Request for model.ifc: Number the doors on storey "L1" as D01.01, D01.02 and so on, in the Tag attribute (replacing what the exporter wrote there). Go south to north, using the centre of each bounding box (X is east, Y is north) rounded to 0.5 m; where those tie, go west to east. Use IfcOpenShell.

First a look at what the model holds.

```python
import ifcopenshell
import ifcopenshell.util.element
import ifcopenshell.util.placement

model = ifcopenshell.open("model.ifc")
print(model.schema)
storey = next(s for s in model.by_type("IfcBuildingStorey") if s.Name == "L1")
doors = [e for e in ifcopenshell.util.element.get_decomposition(storey) if e.is_a("IfcDoor")]
for e in sorted(doors, key=lambda e: e.id()):
    origin = ifcopenshell.util.placement.get_local_placement(e.ObjectPlacement)[:3, 3]
    print(e.id(), e.Tag, e.Name, origin.round(2) + 0.0, sep=" | ")
```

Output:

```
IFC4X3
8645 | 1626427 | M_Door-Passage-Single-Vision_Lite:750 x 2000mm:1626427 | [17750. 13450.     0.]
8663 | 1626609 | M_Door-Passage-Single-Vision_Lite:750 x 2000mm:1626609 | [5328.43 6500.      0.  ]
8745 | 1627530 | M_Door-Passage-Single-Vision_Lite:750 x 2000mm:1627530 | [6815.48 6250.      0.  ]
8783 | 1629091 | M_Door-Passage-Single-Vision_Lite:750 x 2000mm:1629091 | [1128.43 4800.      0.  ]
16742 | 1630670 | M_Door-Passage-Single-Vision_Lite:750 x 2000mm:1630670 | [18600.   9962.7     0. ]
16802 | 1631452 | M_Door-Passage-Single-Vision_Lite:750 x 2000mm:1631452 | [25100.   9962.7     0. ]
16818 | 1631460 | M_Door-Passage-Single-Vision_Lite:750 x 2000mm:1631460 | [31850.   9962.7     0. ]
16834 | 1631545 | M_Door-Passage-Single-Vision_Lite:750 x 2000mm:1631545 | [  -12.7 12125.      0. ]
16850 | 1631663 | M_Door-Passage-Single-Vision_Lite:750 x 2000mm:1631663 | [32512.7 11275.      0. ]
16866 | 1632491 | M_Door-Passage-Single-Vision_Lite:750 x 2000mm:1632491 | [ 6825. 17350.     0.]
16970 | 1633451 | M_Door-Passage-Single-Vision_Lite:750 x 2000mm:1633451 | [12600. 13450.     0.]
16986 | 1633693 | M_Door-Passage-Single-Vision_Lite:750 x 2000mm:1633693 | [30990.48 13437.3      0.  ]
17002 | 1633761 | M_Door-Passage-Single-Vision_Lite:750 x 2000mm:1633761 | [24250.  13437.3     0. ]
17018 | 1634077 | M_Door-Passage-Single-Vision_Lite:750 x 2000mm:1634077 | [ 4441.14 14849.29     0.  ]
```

```python
import ifcopenshell
import ifcopenshell.geom
import ifcopenshell.util.element
import ifcopenshell.util.shape

model = ifcopenshell.open("model.ifc")
settings = ifcopenshell.geom.settings()
settings.set("use-world-coords", True)


def centre(element):
    shape = ifcopenshell.geom.create_shape(settings, element)
    return ifcopenshell.util.shape.get_bbox_centroid(shape.geometry)


storey = next(s for s in model.by_type("IfcBuildingStorey") if s.Name == "L1")
doors = [e for e in ifcopenshell.util.element.get_decomposition(storey) if e.is_a("IfcDoor")]

# Insertion points can sit at a corner or the storey origin, so sort by the geometry (in metres).
centres = {e: centre(e) for e in doors}
doors.sort(key=lambda e: (round(centres[e][1] / 0.5), centres[e][0]))

for i, e in enumerate(doors, start=1):
    number = f"D01.{i:02d}"
    e.Tag = number
    print(e.id(), number)

model.write("model_v2.ifc")
```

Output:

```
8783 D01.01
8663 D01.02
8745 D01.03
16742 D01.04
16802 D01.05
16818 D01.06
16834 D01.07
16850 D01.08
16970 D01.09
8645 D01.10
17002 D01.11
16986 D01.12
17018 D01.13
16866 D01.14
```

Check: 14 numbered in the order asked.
